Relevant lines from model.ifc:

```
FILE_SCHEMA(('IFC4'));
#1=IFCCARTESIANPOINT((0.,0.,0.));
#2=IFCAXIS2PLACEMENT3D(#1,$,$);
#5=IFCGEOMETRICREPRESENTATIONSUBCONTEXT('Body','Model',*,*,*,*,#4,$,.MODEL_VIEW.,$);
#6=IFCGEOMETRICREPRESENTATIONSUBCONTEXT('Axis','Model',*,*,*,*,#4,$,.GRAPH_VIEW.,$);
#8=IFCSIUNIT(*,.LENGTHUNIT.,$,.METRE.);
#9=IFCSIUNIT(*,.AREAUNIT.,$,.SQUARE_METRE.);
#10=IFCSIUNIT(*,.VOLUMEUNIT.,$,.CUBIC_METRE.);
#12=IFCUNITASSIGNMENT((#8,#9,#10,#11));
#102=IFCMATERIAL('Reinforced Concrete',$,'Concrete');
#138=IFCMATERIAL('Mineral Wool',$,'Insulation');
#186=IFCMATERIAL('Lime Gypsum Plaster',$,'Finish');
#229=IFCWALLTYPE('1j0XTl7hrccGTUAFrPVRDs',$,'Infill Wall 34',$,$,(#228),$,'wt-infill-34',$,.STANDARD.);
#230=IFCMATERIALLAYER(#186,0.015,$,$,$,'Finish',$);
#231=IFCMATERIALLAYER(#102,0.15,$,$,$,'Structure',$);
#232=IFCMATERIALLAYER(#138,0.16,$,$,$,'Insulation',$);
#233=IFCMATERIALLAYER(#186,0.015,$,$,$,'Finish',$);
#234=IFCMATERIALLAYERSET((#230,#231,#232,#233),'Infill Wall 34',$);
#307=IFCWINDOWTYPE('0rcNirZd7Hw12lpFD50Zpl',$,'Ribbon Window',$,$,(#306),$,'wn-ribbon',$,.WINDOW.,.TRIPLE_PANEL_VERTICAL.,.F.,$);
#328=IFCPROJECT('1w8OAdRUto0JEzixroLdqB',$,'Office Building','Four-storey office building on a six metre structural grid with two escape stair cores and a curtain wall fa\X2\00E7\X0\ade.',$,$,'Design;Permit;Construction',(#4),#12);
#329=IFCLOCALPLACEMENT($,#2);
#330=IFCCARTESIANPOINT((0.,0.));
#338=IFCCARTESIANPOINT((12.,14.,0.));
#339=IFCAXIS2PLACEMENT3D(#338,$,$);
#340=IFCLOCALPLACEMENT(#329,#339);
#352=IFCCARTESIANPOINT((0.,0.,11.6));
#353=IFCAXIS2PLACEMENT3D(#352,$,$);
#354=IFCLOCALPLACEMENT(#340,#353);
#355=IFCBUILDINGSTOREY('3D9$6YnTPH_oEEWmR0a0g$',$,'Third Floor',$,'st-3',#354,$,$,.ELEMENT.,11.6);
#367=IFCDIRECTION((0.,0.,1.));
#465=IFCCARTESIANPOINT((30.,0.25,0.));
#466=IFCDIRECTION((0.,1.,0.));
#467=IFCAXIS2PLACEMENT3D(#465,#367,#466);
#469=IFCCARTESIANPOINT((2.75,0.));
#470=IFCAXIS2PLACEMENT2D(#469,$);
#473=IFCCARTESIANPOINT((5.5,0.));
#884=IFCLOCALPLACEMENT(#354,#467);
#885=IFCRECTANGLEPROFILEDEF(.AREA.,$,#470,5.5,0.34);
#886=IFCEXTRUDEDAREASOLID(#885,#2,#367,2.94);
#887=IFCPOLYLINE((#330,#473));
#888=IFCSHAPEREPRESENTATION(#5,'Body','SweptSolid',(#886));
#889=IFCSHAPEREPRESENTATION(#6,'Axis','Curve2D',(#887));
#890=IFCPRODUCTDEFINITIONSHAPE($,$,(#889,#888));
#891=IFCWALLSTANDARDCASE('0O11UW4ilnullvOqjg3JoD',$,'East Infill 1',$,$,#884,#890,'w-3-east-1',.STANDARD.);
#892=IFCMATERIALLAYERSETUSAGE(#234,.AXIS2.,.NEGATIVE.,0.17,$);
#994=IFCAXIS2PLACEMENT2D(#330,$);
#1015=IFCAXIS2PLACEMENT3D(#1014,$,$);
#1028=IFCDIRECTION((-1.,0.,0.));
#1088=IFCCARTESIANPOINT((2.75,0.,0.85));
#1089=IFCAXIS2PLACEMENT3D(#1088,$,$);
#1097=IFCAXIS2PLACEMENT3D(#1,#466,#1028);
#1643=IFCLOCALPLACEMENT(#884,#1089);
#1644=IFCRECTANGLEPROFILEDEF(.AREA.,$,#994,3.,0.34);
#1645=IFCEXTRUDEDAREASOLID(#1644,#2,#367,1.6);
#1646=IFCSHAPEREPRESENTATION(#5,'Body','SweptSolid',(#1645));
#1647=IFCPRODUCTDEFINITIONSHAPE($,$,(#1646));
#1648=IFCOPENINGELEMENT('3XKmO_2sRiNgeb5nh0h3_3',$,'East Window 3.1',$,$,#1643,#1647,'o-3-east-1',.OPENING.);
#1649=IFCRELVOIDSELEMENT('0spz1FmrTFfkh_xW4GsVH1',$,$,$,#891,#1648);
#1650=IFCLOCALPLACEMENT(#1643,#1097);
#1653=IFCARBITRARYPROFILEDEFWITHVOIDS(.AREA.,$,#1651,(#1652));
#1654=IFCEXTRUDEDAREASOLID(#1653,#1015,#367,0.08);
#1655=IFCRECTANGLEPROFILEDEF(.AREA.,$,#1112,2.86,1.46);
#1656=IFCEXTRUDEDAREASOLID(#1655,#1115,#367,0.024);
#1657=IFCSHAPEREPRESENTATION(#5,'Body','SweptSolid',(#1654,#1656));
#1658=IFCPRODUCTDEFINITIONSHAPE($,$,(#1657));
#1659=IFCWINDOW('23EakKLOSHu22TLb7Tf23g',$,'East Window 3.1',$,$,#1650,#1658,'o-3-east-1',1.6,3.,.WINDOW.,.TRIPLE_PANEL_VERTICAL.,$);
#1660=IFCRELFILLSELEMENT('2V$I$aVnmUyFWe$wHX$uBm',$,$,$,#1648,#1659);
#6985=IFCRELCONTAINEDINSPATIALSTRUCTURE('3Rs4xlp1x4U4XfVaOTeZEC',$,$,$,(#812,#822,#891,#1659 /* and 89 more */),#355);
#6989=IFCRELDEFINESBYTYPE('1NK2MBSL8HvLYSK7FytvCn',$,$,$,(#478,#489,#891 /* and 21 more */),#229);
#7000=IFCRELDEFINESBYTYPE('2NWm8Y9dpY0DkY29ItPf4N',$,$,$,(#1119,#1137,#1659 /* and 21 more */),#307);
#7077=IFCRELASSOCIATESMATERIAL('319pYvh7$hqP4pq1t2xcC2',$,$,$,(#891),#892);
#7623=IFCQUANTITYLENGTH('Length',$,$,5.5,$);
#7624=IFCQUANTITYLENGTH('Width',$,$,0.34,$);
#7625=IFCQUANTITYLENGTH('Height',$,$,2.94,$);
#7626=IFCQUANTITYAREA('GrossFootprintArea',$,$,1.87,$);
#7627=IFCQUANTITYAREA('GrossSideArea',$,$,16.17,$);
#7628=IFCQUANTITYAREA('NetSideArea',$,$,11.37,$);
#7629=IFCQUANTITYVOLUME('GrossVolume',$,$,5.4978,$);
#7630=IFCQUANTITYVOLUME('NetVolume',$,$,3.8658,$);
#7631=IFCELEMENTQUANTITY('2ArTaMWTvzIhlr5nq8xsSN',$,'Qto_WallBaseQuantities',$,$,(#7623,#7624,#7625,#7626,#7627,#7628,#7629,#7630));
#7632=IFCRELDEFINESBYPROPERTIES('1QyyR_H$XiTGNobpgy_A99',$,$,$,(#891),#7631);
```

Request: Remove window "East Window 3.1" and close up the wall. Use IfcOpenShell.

```python
import ifcopenshell
import ifcopenshell.api.feature
import ifcopenshell.api.pset
import ifcopenshell.api.root
import ifcopenshell.geom
import ifcopenshell.util.element
import ifcopenshell.util.shape
import ifcopenshell.util.unit

model = ifcopenshell.open("model.ifc")
area_scale = ifcopenshell.util.unit.calculate_unit_scale(model, "AREAUNIT")
volume_scale = ifcopenshell.util.unit.calculate_unit_scale(model, "VOLUMEUNIT")
settings = ifcopenshell.geom.settings()


def volume(element):
    """Net volume in cubic metres, openings subtracted."""
    shape = ifcopenshell.geom.create_shape(settings, element)
    return ifcopenshell.util.shape.get_volume(shape.geometry)


window = model.by_guid("23EakKLOSHu22TLb7Tf23g")
opening = window.FillsVoids[0].RelatingOpeningElement
wall = opening.VoidsElements[0].RelatingBuildingElement
before = volume(wall)

ifcopenshell.api.root.remove_product(model, product=window)
ifcopenshell.api.feature.remove_feature(model, feature=opening)

after = volume(wall)
thickness = 0.34  # wall thickness in metres

# Update the wall's stored quantities.
qto = model.by_id(ifcopenshell.util.element.get_pset(wall, "Qto_WallBaseQuantities", should_inherit=False)["id"])
ifcopenshell.api.pset.edit_qto(model, qto=qto, properties={
    "NetSideArea": after / thickness / area_scale,
    "NetVolume": after / volume_scale,
})

print(f"wall volume {before:.3f} -> {after:.3f} m3")

model.write("model_edited.ifc")
```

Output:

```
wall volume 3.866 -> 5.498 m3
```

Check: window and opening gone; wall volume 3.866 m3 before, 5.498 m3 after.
